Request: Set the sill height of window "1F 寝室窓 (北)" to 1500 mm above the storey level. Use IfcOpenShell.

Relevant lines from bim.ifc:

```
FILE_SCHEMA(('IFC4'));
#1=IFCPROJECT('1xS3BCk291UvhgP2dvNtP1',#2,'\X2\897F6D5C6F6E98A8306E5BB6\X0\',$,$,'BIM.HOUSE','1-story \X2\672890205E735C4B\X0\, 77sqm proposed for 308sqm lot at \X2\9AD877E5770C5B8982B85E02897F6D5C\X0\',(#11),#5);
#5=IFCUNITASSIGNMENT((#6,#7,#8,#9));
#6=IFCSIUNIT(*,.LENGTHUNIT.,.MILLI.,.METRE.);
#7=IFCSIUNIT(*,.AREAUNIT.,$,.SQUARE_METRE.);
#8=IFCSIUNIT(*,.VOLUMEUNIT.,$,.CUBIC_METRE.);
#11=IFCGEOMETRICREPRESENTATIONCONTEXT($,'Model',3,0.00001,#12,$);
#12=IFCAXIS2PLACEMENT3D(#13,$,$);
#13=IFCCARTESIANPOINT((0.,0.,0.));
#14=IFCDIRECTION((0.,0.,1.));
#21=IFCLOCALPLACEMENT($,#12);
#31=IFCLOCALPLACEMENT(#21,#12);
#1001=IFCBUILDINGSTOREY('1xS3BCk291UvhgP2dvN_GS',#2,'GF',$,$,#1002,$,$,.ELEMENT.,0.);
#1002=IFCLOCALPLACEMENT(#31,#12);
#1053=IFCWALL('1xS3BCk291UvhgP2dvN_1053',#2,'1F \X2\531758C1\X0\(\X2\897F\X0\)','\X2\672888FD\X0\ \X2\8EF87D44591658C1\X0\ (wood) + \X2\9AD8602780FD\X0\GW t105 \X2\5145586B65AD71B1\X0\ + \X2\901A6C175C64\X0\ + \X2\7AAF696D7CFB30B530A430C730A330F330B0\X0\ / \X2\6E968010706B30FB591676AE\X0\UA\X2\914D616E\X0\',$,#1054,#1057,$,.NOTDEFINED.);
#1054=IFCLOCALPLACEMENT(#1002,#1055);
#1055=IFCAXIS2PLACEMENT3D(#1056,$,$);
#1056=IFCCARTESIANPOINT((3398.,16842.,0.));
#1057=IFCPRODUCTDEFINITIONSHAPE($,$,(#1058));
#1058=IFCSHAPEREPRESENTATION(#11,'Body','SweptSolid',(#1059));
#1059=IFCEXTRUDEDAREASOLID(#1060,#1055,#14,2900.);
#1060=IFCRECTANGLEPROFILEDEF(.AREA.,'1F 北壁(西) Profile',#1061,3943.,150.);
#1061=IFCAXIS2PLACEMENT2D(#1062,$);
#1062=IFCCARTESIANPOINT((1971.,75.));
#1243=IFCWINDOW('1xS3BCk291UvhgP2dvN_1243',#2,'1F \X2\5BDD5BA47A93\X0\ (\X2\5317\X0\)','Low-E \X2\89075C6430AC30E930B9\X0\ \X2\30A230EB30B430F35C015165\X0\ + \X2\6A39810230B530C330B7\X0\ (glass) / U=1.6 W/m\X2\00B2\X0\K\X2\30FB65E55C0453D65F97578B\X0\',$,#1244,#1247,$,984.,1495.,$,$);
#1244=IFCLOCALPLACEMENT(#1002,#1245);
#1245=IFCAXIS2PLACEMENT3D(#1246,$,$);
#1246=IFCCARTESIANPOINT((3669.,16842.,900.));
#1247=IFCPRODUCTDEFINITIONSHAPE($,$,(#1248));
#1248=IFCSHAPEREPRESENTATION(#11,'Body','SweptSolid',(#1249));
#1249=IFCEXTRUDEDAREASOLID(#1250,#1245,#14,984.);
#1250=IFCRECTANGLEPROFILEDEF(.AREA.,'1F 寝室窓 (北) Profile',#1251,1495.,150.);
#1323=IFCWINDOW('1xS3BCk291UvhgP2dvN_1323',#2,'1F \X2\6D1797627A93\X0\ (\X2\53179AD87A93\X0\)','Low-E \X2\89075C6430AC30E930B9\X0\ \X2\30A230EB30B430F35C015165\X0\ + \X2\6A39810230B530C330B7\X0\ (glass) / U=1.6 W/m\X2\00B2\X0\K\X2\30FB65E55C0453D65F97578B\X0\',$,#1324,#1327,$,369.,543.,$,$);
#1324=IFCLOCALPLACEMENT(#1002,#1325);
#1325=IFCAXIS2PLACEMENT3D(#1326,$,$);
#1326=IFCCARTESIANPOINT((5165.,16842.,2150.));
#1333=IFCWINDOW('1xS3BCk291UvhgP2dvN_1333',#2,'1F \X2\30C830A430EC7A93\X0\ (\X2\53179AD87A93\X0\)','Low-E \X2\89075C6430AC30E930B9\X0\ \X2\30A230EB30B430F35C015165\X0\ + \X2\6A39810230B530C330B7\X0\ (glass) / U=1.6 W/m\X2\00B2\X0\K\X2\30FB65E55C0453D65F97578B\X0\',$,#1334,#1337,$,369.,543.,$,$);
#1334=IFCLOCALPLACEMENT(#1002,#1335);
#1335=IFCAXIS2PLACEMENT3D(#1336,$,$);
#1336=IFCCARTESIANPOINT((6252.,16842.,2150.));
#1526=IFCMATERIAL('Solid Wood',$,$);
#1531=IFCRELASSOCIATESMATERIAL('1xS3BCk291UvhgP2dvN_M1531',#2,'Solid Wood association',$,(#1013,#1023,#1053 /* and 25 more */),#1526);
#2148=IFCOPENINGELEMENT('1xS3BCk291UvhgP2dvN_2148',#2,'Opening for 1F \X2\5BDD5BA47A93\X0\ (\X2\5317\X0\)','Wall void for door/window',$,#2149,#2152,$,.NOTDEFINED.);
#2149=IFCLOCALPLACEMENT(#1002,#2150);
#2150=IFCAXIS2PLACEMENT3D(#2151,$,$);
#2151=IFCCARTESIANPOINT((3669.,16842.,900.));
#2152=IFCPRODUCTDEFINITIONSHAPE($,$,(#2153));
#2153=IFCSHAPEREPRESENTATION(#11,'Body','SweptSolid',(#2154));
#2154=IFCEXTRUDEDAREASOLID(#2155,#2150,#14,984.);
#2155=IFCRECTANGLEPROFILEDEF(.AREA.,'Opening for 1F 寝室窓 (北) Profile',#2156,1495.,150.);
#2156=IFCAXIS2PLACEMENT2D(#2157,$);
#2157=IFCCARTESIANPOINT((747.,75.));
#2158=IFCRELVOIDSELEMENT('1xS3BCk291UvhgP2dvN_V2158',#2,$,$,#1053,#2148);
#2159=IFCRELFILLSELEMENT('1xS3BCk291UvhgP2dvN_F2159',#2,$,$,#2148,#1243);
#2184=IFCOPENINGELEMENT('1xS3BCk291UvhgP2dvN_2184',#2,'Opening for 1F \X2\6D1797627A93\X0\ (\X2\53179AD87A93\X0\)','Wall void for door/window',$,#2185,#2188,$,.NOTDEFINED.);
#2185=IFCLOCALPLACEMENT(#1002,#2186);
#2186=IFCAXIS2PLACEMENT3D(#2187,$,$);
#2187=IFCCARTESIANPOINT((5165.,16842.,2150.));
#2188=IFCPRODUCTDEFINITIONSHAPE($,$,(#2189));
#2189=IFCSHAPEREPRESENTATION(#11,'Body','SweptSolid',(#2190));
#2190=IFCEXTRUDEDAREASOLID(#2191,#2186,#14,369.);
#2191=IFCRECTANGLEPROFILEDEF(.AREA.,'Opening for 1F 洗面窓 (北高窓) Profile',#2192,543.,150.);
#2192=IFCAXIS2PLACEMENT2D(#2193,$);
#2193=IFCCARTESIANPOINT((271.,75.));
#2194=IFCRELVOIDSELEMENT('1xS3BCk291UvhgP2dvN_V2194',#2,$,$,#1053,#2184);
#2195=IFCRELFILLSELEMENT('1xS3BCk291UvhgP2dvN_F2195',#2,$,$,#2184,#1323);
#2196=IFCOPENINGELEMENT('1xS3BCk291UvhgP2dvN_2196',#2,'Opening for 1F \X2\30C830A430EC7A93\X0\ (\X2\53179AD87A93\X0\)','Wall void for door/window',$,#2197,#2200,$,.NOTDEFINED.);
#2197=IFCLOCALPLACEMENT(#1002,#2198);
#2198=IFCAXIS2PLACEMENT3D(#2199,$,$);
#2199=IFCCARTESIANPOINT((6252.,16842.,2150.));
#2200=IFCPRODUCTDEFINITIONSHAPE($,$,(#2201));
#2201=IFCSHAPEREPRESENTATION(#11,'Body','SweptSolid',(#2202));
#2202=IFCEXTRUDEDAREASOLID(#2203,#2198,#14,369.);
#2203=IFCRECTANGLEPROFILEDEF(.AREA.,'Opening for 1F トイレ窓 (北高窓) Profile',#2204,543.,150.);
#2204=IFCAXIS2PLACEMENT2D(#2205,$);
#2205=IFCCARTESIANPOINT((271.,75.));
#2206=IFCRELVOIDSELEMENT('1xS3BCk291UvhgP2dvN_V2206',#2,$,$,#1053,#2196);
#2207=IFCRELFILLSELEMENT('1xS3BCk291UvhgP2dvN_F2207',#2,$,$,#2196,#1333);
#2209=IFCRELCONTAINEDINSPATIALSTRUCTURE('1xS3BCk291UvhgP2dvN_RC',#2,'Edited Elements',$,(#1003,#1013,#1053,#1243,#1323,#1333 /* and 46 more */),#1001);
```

```python
import numpy as np
import ifcopenshell
import ifcopenshell.api.geometry
import ifcopenshell.geom
import ifcopenshell.util.element
import ifcopenshell.util.placement
import ifcopenshell.util.shape
import ifcopenshell.util.unit

model = ifcopenshell.open("bim.ifc")
unit_scale = ifcopenshell.util.unit.calculate_unit_scale(model)

window = model.by_guid("1xS3BCk291UvhgP2dvN_1243")
opening = window.FillsVoids[0].RelatingOpeningElement
storey = ifcopenshell.util.element.get_container(window, ifc_class="IfcBuildingStorey")
level = ifcopenshell.util.placement.get_local_placement(storey.ObjectPlacement)[2, 3]

# The opening's origin need not be at the sill, so measure its lowest point.
shape = ifcopenshell.geom.create_shape(ifcopenshell.geom.settings(), opening)
bottom = ifcopenshell.util.shape.get_shape_bottom_elevation(shape, shape.geometry) / unit_scale
dz = level + 1500.0 - bottom

shift = np.array([0.0, 0.0, dz])
# The window is not placed relative to its opening, so move both.
for product in (opening, window):
    matrix = ifcopenshell.util.placement.get_local_placement(product.ObjectPlacement)
    matrix[:3, 3] += shift
    ifcopenshell.api.geometry.edit_object_placement(model, product=product, matrix=matrix, is_si=False)

print(f"moved by {dz * unit_scale:+.3f} m")

model.write("bim_v2.ifc")
```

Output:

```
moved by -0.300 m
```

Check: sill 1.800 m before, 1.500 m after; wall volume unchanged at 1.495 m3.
